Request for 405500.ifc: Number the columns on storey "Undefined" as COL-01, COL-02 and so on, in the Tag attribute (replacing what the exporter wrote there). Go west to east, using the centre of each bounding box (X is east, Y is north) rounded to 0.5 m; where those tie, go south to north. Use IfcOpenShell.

First a look at what the model holds.

```python
import ifcopenshell
import ifcopenshell.util.element
import ifcopenshell.util.placement

model = ifcopenshell.open("405500.ifc")
print(model.schema)
storey = next(s for s in model.by_type("IfcBuildingStorey") if s.Name == "Undefined")
columns = [e for e in ifcopenshell.util.element.get_decomposition(storey) if e.is_a("IfcColumn")]
for e in sorted(columns, key=lambda e: e.id()):
    origin = ifcopenshell.util.placement.get_local_placement(e.ObjectPlacement)[:3, 3]
    print(e.id(), e.Tag, e.Name, origin.round(2) + 0.0, sep=" | ")
```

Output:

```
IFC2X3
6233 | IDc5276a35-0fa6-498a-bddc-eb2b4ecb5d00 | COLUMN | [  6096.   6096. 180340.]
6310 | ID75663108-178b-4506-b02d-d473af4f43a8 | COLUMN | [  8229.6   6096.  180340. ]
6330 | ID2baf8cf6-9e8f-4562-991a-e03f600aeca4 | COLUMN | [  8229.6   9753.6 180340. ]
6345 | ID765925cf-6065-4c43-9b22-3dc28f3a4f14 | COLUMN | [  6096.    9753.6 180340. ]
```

```python
import ifcopenshell
import ifcopenshell.geom
import ifcopenshell.util.element
import ifcopenshell.util.shape

model = ifcopenshell.open("405500.ifc")
settings = ifcopenshell.geom.settings()
settings.set("use-world-coords", True)


def centre(element):
    shape = ifcopenshell.geom.create_shape(settings, element)
    return ifcopenshell.util.shape.get_bbox_centroid(shape.geometry)


storey = next(s for s in model.by_type("IfcBuildingStorey") if s.Name == "Undefined")
columns = [e for e in ifcopenshell.util.element.get_decomposition(storey) if e.is_a("IfcColumn")]

# Insertion points can sit at a corner or the storey origin, so sort by the geometry (in metres).
centres = {e: centre(e) for e in columns}
columns.sort(key=lambda e: (round(centres[e][0] / 0.5), centres[e][1]))

for i, e in enumerate(columns, start=1):
    number = f"COL-{i:02d}"
    e.Tag = number
    print(e.id(), number)

model.write("405500_v2.ifc")
```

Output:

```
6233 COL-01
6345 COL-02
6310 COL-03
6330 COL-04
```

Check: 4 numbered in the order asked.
